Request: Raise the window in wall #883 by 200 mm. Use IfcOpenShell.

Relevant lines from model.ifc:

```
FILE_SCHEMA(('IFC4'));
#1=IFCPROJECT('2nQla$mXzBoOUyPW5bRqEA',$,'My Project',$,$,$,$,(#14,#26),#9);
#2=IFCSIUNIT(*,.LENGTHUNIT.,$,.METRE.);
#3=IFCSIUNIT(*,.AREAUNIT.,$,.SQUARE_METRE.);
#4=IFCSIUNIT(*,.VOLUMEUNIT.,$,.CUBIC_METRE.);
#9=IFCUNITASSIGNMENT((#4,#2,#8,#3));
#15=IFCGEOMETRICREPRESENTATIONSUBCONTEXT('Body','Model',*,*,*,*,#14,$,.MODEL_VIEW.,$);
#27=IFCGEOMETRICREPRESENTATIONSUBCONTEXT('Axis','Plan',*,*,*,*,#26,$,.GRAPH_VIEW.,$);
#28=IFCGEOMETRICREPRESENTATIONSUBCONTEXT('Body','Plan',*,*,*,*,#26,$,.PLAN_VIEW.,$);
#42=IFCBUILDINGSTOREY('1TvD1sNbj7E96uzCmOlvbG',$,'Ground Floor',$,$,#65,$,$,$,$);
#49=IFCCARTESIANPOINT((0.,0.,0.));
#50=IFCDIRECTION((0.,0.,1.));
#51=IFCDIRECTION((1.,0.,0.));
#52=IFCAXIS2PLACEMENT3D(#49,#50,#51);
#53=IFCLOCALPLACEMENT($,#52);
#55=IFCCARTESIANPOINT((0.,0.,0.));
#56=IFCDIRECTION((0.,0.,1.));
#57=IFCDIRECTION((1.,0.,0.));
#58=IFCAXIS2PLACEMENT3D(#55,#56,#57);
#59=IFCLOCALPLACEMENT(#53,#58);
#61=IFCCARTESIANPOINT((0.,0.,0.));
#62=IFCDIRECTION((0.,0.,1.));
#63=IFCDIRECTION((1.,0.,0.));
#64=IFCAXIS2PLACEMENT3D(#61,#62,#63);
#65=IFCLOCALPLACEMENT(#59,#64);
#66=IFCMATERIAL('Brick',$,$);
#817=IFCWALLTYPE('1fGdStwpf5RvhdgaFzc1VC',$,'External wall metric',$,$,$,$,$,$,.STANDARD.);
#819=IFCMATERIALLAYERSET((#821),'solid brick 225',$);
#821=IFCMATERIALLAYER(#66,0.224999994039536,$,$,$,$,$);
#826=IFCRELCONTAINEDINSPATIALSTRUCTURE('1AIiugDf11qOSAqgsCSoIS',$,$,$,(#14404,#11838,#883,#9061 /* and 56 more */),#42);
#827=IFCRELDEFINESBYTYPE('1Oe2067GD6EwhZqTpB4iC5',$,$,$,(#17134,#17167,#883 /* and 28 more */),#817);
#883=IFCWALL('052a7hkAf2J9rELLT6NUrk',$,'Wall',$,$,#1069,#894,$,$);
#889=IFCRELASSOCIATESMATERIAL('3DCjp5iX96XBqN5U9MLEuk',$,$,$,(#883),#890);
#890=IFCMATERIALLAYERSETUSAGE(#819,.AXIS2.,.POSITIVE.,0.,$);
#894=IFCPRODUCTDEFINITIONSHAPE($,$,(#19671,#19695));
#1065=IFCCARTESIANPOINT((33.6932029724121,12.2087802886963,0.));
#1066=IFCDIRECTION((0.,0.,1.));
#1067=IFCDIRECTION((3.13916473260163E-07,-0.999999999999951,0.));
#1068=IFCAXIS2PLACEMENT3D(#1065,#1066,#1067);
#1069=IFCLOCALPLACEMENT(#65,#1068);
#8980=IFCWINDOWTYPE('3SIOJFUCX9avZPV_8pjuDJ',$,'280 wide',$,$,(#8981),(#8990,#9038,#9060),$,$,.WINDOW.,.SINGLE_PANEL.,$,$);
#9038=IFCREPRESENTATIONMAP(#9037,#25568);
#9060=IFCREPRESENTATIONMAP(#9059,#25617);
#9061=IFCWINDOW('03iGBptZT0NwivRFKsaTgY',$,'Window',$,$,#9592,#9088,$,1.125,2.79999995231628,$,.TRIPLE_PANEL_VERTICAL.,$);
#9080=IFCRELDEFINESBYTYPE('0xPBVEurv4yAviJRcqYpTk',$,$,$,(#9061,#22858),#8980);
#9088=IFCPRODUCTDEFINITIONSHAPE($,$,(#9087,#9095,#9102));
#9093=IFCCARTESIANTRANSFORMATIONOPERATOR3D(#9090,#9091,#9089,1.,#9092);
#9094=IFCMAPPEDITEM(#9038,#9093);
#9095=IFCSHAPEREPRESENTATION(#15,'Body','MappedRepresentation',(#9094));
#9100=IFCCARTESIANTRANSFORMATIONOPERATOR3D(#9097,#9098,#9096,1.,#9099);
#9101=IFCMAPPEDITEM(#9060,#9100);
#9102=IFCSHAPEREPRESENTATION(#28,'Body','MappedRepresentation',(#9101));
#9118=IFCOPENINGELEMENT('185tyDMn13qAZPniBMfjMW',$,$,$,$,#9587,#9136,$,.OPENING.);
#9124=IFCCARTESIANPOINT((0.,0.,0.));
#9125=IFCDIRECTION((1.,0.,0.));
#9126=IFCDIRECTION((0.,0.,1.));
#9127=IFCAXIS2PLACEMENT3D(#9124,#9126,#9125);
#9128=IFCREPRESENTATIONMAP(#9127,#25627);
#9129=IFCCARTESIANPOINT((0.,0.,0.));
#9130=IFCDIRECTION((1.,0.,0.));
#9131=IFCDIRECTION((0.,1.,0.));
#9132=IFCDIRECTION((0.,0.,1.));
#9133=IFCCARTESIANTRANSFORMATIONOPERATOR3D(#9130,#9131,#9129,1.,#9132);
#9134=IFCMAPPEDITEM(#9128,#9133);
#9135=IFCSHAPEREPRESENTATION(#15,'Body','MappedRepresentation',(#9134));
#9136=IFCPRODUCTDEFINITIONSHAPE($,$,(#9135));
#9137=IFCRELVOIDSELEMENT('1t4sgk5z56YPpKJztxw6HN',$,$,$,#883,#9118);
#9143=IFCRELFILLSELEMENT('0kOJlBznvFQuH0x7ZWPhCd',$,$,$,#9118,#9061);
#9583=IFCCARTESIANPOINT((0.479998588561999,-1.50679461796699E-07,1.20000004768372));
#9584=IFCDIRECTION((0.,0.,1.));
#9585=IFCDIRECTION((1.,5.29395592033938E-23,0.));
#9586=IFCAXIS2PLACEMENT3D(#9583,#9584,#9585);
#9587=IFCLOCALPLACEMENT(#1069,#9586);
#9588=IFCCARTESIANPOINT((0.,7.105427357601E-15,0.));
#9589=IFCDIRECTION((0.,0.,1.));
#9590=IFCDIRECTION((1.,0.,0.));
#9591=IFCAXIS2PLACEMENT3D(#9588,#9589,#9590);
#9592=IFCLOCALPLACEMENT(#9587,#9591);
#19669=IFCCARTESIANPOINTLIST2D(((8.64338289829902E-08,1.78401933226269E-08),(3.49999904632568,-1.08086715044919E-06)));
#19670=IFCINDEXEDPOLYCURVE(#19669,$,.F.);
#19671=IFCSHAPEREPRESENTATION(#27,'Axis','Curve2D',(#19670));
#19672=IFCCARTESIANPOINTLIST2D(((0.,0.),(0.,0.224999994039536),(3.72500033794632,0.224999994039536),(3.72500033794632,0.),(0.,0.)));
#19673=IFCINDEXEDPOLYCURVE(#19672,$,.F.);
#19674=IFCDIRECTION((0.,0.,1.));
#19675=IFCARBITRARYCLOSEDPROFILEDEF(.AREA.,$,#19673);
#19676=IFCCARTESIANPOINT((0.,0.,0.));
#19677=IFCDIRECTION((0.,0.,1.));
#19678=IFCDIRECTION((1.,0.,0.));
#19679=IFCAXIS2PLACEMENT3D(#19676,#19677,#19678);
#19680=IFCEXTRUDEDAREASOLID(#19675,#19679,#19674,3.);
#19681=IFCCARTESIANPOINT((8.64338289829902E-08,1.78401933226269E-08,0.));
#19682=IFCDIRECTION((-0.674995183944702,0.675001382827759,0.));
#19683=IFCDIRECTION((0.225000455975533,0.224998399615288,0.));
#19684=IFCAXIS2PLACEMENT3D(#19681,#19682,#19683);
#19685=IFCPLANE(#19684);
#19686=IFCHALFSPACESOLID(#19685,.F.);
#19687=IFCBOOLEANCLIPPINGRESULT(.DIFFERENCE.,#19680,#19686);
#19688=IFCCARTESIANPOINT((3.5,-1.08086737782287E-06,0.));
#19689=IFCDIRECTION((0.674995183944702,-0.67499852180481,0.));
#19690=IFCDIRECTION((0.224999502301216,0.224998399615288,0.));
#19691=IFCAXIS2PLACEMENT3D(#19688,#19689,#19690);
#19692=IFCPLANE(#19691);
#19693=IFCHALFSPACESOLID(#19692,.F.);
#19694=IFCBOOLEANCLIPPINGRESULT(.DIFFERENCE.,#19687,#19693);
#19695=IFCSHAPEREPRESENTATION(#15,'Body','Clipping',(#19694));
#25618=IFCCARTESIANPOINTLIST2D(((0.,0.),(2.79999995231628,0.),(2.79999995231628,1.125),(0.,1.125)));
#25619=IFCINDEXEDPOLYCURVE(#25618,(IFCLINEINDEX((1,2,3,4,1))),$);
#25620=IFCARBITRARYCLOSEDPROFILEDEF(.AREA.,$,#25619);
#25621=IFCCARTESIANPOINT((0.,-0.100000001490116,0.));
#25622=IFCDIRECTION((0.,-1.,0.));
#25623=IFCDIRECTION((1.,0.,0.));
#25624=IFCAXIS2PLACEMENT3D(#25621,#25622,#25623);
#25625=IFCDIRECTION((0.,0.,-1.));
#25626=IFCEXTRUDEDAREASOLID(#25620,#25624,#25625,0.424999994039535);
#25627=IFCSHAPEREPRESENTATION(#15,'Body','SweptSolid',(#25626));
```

```python
import numpy as np
import ifcopenshell
import ifcopenshell.api.geometry
import ifcopenshell.util.placement
import ifcopenshell.util.unit

model = ifcopenshell.open("model.ifc")
unit_scale = ifcopenshell.util.unit.calculate_unit_scale(model)

window = model.by_guid("03iGBptZT0NwivRFKsaTgY")
opening = window.FillsVoids[0].RelatingOpeningElement
dz = 0.2 / unit_scale

shift = np.array([0.0, 0.0, dz])
# The window is placed relative to its opening, so it follows when the opening moves.
matrix = ifcopenshell.util.placement.get_local_placement(opening.ObjectPlacement)
matrix[:3, 3] += shift
ifcopenshell.api.geometry.edit_object_placement(
    model, product=opening, matrix=matrix, is_si=False, should_transform_children=True
)

print(f"moved by {dz * unit_scale:+.3f} m")

model.write("model_edited.ifc")
```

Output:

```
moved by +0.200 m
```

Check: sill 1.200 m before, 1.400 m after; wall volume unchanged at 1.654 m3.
